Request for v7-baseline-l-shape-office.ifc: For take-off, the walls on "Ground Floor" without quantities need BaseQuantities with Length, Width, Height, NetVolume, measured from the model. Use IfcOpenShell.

First a look at what the model holds.

```python
import ifcopenshell
import ifcopenshell.util.element
import ifcopenshell.util.unit

model = ifcopenshell.open("v7-baseline-l-shape-office.ifc")
print(model.schema)
for unit_type in ("LENGTHUNIT", "AREAUNIT", "VOLUMEUNIT"):
    print(unit_type, ifcopenshell.util.unit.calculate_unit_scale(model, unit_type))
storey = next(s for s in model.by_type("IfcBuildingStorey") if s.Name == "Ground Floor")
walls = [e for e in ifcopenshell.util.element.get_decomposition(storey) if e.is_a("IfcWall")]
for e in sorted(walls, key=lambda e: e.id()):
    print(e.id(), e.is_a(), e.Name, list(ifcopenshell.util.element.get_psets(e, qtos_only=True)), sep=" | ")
```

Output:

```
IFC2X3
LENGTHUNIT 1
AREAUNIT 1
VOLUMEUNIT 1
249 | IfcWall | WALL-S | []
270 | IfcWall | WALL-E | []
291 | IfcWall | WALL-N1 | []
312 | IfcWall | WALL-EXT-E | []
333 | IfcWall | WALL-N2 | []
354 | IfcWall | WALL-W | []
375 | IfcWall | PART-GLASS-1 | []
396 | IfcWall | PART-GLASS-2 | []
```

```python
import ifcopenshell
import ifcopenshell.api.pset
import ifcopenshell.geom
import ifcopenshell.util.element
import ifcopenshell.util.shape
import ifcopenshell.util.unit

model = ifcopenshell.open("v7-baseline-l-shape-office.ifc")
unit_scale = ifcopenshell.util.unit.calculate_unit_scale(model)
volume_scale = ifcopenshell.util.unit.calculate_unit_scale(model, "VOLUMEUNIT")
settings = ifcopenshell.geom.settings()

storey = next(s for s in model.by_type("IfcBuildingStorey") if s.Name == "Ground Floor")
walls = [e for e in ifcopenshell.util.element.get_decomposition(storey) if e.is_a("IfcWall")]

for e in sorted(walls, key=lambda e: e.id()):
    if ifcopenshell.util.element.get_psets(e, qtos_only=True, should_inherit=False):
        continue
    # Geometry comes back in metres, in the element's own axes.
    shape = ifcopenshell.geom.create_shape(settings, e)
    values = {
        "Length": ifcopenshell.util.shape.get_x(shape.geometry) / unit_scale,
        "Width": ifcopenshell.util.shape.get_y(shape.geometry) / unit_scale,
        "Height": ifcopenshell.util.shape.get_z(shape.geometry) / unit_scale,
        "NetVolume": ifcopenshell.util.shape.get_volume(shape.geometry) / volume_scale,
    }
    qto = ifcopenshell.api.pset.add_qto(model, product=e, name="BaseQuantities")
    ifcopenshell.api.pset.edit_qto(model, qto=qto, properties=values)
    print(e.id(), {k: round(v, 3) for k, v in values.items()})

model.write("v7-baseline-l-shape-office_updated.ifc")
```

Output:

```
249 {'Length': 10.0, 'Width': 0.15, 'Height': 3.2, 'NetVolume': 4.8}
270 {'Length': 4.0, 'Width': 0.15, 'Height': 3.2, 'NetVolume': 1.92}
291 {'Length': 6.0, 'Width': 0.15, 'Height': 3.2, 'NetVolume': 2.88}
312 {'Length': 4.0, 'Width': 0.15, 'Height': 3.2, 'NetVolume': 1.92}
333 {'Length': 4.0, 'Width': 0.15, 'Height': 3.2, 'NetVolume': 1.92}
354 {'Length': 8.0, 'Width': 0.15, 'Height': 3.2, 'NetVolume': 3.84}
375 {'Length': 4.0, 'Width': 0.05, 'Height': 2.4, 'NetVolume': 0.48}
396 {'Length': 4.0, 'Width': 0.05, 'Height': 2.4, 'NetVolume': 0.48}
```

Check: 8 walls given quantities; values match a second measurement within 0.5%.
